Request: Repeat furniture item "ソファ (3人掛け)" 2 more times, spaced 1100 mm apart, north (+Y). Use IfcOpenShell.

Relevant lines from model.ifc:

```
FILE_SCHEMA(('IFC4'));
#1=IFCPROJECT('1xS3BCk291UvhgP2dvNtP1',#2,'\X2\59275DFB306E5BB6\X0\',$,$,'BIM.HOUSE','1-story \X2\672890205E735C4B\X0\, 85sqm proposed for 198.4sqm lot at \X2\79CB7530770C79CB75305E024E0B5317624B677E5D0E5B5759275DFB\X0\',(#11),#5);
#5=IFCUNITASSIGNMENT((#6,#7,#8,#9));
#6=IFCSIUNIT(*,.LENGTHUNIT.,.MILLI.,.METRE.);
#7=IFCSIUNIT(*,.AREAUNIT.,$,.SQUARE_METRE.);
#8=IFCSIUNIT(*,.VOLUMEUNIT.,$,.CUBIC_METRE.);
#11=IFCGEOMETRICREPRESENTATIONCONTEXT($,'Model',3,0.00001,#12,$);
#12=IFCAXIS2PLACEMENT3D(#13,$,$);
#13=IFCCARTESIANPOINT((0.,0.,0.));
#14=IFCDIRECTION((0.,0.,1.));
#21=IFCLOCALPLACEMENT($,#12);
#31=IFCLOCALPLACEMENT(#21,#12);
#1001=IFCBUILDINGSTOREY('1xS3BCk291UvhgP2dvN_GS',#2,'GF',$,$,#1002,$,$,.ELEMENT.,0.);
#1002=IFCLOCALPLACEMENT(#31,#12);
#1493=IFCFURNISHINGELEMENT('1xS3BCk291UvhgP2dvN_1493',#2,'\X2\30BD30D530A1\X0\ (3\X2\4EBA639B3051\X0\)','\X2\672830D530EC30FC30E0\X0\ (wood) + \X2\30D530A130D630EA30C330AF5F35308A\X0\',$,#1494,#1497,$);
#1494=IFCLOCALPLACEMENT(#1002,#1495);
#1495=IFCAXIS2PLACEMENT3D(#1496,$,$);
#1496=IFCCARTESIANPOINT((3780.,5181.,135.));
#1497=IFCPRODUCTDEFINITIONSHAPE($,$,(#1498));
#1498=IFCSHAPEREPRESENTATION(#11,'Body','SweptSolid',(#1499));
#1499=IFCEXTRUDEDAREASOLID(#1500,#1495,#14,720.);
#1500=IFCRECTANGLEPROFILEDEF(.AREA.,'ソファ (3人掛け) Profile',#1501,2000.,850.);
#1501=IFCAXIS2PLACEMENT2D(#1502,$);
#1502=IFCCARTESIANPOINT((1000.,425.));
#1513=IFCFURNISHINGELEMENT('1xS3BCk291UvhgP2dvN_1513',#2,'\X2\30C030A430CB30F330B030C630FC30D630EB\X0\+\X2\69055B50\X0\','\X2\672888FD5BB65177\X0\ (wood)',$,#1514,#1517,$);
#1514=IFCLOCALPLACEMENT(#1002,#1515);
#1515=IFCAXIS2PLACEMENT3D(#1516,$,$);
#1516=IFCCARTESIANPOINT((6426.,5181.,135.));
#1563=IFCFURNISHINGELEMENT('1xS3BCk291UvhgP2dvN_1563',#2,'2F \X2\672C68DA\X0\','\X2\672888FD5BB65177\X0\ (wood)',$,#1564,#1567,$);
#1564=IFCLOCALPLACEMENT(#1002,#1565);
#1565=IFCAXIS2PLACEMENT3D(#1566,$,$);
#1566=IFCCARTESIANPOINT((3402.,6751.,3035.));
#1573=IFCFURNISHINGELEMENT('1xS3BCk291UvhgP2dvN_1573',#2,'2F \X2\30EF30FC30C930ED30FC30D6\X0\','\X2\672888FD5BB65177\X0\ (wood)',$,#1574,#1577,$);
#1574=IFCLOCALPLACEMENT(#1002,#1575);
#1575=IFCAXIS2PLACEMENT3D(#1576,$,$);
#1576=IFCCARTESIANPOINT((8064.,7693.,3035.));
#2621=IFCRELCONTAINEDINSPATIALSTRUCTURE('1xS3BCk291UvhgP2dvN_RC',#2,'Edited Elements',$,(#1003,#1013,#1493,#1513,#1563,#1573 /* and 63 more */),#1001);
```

```python
import numpy as np
import ifcopenshell
import ifcopenshell.api.geometry
import ifcopenshell.api.root
import ifcopenshell.util.element
import ifcopenshell.util.placement
import ifcopenshell.util.unit

model = ifcopenshell.open("model.ifc")
unit_scale = ifcopenshell.util.unit.calculate_unit_scale(model)


def reuse_history(source, copy):
    """copy_class also copies each property set's owner history, people and application; keep the originals."""
    for rel in copy.IsDefinedBy:
        if rel.is_a("IfcRelDefinesByProperties") and (history := rel.RelatingPropertyDefinition.OwnerHistory):
            rel.RelatingPropertyDefinition.OwnerHistory = source.OwnerHistory
            ifcopenshell.util.element.remove_deep2(model, history)


source = model.by_guid("1xS3BCk291UvhgP2dvN_1493")
base = ifcopenshell.util.placement.get_local_placement(source.ObjectPlacement)
step = np.array([0.0, 1.0, 0.0]) * 1.1 / unit_scale

for i in range(1, 3):
    copy = ifcopenshell.api.root.copy_class(model, product=source)
    copy.Representation = ifcopenshell.util.element.copy_deep(
        model, source.Representation, exclude=["IfcGeometricRepresentationContext", "IfcRepresentationMap"]
    )
    reuse_history(source, copy)
    matrix = base.copy()
    matrix[:3, 3] += i * step
    print("added at", matrix[:3, 3].round(3) + 0.0)
    ifcopenshell.api.geometry.edit_object_placement(model, product=copy, matrix=matrix, is_si=False)

model.write("model_edited.ifc")
```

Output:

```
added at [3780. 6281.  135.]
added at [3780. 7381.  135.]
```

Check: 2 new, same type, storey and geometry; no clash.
